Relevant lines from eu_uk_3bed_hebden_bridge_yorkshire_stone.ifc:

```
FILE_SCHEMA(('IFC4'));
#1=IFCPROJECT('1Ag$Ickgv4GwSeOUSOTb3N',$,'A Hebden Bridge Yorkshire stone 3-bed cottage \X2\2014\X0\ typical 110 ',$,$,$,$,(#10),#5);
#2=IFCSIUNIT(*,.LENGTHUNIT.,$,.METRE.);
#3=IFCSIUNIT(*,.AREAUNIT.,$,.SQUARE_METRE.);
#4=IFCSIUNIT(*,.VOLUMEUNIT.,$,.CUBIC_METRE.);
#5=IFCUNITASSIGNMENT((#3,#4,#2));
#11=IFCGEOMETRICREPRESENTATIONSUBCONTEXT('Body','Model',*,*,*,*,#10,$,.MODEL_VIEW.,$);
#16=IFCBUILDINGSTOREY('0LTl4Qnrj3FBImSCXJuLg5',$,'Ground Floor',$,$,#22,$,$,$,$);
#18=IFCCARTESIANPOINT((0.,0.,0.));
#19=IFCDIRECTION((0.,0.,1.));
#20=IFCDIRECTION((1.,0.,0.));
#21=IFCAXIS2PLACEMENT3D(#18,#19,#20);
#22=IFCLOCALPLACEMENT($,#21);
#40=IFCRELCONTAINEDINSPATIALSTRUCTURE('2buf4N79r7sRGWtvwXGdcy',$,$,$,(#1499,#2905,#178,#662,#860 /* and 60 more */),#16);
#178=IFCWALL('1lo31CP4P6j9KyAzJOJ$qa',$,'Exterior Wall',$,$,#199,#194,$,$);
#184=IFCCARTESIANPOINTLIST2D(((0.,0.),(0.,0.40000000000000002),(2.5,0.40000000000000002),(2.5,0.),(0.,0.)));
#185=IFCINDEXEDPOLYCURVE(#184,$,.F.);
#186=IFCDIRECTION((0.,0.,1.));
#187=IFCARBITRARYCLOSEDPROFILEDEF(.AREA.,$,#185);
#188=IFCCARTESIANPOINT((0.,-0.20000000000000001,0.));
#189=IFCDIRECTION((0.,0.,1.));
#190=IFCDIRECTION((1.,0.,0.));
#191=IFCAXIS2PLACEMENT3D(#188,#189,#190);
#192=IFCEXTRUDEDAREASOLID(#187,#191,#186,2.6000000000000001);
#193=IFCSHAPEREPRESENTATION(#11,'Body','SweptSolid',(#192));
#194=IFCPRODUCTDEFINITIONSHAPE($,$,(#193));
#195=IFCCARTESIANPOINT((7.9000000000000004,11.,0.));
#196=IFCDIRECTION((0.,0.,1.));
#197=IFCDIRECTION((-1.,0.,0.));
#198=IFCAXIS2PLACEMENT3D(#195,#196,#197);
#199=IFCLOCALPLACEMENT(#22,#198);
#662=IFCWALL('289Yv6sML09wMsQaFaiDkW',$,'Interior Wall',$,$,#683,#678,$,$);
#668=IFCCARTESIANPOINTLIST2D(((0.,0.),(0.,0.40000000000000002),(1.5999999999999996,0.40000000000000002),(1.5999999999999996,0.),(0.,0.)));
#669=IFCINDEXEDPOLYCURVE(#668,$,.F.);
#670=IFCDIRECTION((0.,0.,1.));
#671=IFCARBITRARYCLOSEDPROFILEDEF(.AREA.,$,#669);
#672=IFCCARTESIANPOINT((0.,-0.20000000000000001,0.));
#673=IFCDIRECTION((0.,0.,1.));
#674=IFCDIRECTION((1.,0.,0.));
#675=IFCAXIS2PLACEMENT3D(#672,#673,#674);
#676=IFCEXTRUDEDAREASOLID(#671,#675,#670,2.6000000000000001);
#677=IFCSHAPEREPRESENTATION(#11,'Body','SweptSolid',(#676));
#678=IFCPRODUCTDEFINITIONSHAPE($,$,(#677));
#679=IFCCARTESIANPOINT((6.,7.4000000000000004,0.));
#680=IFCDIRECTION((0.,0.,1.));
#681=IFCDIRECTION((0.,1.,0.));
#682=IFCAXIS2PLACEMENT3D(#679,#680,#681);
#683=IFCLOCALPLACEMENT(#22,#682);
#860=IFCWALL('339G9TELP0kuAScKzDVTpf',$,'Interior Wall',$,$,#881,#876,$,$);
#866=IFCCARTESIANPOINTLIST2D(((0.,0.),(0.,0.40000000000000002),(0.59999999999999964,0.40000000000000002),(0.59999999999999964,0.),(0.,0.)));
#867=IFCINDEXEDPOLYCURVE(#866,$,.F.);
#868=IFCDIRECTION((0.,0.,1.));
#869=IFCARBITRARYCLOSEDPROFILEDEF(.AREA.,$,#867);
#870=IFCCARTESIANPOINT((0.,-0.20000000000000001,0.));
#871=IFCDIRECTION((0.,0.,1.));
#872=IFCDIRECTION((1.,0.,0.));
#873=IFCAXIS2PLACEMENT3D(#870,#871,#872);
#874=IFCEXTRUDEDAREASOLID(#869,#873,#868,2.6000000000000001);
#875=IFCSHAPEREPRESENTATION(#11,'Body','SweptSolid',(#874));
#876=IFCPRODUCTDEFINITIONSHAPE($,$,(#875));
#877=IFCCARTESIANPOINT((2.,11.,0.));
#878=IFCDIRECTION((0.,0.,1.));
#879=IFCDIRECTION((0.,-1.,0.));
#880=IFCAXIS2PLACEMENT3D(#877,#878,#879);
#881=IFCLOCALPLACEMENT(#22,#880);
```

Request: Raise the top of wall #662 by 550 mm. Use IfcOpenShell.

```python
import ifcopenshell
import ifcopenshell.geom
import ifcopenshell.util.representation
import ifcopenshell.util.shape
import ifcopenshell.util.unit

model = ifcopenshell.open("eu_uk_3bed_hebden_bridge_yorkshire_stone.ifc")
unit_scale = ifcopenshell.util.unit.calculate_unit_scale(model)
settings = ifcopenshell.geom.settings()


def volume(element):
    """Net volume in cubic metres, openings subtracted."""
    shape = ifcopenshell.geom.create_shape(settings, element)
    return ifcopenshell.util.shape.get_volume(shape.geometry)


wall = model.by_guid("289Yv6sML09wMsQaFaiDkW")
before = volume(wall)

body = ifcopenshell.util.representation.get_representation(wall, "Model", "Body")
solid = body.Items[0]
old_height = solid.Depth
solid.Depth += 0.55 / unit_scale
after = volume(wall)

print(f"height {old_height:g} -> {solid.Depth:g}, volume {before:.3f} -> {after:.3f} m3")

model.write("eu_uk_3bed_hebden_bridge_yorkshire_stone_updated.ifc")
```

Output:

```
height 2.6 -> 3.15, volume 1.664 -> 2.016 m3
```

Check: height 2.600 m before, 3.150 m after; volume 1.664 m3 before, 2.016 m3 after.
